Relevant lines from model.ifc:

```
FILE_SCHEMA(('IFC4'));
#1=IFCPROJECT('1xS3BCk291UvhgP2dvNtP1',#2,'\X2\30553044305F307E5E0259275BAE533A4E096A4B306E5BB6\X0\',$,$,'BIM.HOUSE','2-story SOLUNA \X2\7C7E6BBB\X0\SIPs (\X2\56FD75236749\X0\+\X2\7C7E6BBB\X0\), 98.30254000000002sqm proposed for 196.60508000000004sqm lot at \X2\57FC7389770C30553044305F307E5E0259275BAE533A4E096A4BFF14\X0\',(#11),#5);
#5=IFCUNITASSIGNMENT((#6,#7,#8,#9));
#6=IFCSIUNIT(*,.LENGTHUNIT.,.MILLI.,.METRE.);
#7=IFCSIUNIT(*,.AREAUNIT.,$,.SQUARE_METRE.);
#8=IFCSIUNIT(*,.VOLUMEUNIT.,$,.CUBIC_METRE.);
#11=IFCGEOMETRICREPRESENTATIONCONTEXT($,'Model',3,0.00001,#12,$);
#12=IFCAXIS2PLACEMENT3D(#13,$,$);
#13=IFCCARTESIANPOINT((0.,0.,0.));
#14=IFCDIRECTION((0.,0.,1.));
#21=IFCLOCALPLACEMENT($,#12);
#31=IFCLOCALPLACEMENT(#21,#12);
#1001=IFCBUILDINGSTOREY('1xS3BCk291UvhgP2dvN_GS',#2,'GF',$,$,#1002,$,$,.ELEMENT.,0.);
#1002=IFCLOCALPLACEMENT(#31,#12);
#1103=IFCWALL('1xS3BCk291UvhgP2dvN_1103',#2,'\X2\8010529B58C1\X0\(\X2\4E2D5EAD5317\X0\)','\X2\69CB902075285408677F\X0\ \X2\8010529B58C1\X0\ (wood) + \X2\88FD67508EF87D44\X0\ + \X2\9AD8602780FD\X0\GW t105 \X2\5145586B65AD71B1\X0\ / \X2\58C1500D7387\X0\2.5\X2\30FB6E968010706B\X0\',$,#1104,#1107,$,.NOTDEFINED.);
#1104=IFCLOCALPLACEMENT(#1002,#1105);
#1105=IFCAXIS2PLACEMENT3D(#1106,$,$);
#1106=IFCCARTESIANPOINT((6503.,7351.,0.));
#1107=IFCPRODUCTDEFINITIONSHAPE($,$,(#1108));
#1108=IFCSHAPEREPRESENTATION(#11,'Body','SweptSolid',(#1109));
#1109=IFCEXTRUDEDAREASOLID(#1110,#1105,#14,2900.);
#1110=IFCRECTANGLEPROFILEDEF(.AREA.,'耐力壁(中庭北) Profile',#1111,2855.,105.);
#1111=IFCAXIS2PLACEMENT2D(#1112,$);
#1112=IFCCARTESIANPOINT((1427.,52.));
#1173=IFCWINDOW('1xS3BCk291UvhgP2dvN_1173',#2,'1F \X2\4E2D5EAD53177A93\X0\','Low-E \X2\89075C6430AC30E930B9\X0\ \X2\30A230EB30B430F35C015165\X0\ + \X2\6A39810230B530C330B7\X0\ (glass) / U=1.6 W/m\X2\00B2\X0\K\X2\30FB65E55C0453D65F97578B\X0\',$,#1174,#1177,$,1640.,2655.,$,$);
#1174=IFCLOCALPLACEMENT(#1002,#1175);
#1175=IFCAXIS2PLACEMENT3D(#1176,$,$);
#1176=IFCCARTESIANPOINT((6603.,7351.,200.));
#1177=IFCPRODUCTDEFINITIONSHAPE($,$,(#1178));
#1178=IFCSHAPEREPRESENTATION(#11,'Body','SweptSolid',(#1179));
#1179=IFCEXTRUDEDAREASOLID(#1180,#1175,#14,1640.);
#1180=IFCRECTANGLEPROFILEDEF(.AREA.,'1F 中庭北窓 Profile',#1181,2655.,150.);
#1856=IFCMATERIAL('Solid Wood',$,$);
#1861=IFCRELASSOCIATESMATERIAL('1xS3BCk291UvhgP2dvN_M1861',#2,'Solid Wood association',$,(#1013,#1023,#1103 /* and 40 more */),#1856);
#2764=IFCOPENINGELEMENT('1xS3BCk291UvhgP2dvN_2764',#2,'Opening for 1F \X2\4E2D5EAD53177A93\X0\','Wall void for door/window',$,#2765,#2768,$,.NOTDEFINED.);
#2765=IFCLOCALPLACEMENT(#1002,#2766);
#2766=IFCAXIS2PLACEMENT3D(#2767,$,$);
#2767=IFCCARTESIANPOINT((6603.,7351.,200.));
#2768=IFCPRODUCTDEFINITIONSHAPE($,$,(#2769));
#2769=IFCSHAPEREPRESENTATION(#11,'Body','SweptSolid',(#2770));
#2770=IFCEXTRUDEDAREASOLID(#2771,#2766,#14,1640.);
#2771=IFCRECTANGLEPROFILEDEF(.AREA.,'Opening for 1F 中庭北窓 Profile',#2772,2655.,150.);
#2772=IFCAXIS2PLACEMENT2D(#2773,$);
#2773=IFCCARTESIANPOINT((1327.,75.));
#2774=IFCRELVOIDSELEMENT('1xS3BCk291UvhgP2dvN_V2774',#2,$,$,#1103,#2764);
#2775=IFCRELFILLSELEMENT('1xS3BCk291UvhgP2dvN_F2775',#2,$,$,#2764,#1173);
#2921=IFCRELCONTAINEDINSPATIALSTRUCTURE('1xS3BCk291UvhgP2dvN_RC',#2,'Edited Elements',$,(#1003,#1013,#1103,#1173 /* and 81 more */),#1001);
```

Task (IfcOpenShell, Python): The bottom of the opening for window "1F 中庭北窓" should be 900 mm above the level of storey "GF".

```python
import numpy as np
import ifcopenshell
import ifcopenshell.api.geometry
import ifcopenshell.geom
import ifcopenshell.util.element
import ifcopenshell.util.placement
import ifcopenshell.util.shape
import ifcopenshell.util.unit

model = ifcopenshell.open("model.ifc")
unit_scale = ifcopenshell.util.unit.calculate_unit_scale(model)

window = model.by_guid("1xS3BCk291UvhgP2dvN_1173")
opening = window.FillsVoids[0].RelatingOpeningElement
storey = ifcopenshell.util.element.get_container(window, ifc_class="IfcBuildingStorey")
level = ifcopenshell.util.placement.get_local_placement(storey.ObjectPlacement)[2, 3]

# The opening's origin need not be at the sill, so measure its lowest point.
shape = ifcopenshell.geom.create_shape(ifcopenshell.geom.settings(), opening)
bottom = ifcopenshell.util.shape.get_shape_bottom_elevation(shape, shape.geometry) / unit_scale
dz = level + 0.9 / unit_scale - bottom

shift = np.array([0.0, 0.0, dz])
# The window is not placed relative to its opening, so move both.
for product in (opening, window):
    matrix = ifcopenshell.util.placement.get_local_placement(product.ObjectPlacement)
    matrix[:3, 3] += shift
    ifcopenshell.api.geometry.edit_object_placement(model, product=product, matrix=matrix, is_si=False)

print(f"moved by {dz * unit_scale:+.3f} m")

model.write("model_edited.ifc")
```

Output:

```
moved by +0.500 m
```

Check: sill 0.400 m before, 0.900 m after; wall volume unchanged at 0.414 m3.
